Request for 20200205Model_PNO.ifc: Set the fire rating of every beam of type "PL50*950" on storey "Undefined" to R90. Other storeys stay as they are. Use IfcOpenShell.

First a look at what the model holds.

```python
import ifcopenshell
import ifcopenshell.util.element

model = ifcopenshell.open("20200205Model_PNO.ifc")
print(model.schema)
storey = next(s for s in model.by_type("IfcBuildingStorey") if s.Name == "Undefined")
beams = [e for e in ifcopenshell.util.element.get_decomposition(storey) if e.is_a("IfcBeam")]
seen = {}
for e in beams:
    element_type = ifcopenshell.util.element.get_type(e)
    key = (element_type.Name if element_type != e and element_type else None, ifcopenshell.util.element.get_pset(e, "Pset_BeamCommon", "FireRating"))
    seen[key] = seen.get(key, 0) + 1
for (name, value), count in sorted(seen.items(), key=str):
    print(count, "x", name, "|", value)
```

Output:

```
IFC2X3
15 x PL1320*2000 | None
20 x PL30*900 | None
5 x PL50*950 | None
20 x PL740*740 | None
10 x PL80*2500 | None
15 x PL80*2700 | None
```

```python
import ifcopenshell
import ifcopenshell.api.pset
import ifcopenshell.util.element

model = ifcopenshell.open("20200205Model_PNO.ifc")

storey = next(s for s in model.by_type("IfcBuildingStorey") if s.Name == "Undefined")
beams = [e for e in ifcopenshell.util.element.get_decomposition(storey) if e.is_a("IfcBeam")]

count = 0
for e in beams:
    element_type = ifcopenshell.util.element.get_type(e)
    if element_type in (None, e) or element_type.Name != "PL50*950":
        continue
    found = ifcopenshell.util.element.get_pset(e, "Pset_BeamCommon", should_inherit=False)
    if found:
        pset = model.by_id(found["id"])
        if len(ifcopenshell.util.element.get_elements_by_pset(pset)) > 1:
            pset = ifcopenshell.api.pset.unshare_pset(model, products=[e], pset=pset)[0]
    else:
        pset = ifcopenshell.api.pset.add_pset(model, product=e, name="Pset_BeamCommon")
    ifcopenshell.api.pset.edit_pset(model, pset=pset, properties={"FireRating": "R90"})
    count += 1

print(count, "beams updated")

model.write("20200205Model_PNO_edited.ifc")
```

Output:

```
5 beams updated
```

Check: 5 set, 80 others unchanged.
